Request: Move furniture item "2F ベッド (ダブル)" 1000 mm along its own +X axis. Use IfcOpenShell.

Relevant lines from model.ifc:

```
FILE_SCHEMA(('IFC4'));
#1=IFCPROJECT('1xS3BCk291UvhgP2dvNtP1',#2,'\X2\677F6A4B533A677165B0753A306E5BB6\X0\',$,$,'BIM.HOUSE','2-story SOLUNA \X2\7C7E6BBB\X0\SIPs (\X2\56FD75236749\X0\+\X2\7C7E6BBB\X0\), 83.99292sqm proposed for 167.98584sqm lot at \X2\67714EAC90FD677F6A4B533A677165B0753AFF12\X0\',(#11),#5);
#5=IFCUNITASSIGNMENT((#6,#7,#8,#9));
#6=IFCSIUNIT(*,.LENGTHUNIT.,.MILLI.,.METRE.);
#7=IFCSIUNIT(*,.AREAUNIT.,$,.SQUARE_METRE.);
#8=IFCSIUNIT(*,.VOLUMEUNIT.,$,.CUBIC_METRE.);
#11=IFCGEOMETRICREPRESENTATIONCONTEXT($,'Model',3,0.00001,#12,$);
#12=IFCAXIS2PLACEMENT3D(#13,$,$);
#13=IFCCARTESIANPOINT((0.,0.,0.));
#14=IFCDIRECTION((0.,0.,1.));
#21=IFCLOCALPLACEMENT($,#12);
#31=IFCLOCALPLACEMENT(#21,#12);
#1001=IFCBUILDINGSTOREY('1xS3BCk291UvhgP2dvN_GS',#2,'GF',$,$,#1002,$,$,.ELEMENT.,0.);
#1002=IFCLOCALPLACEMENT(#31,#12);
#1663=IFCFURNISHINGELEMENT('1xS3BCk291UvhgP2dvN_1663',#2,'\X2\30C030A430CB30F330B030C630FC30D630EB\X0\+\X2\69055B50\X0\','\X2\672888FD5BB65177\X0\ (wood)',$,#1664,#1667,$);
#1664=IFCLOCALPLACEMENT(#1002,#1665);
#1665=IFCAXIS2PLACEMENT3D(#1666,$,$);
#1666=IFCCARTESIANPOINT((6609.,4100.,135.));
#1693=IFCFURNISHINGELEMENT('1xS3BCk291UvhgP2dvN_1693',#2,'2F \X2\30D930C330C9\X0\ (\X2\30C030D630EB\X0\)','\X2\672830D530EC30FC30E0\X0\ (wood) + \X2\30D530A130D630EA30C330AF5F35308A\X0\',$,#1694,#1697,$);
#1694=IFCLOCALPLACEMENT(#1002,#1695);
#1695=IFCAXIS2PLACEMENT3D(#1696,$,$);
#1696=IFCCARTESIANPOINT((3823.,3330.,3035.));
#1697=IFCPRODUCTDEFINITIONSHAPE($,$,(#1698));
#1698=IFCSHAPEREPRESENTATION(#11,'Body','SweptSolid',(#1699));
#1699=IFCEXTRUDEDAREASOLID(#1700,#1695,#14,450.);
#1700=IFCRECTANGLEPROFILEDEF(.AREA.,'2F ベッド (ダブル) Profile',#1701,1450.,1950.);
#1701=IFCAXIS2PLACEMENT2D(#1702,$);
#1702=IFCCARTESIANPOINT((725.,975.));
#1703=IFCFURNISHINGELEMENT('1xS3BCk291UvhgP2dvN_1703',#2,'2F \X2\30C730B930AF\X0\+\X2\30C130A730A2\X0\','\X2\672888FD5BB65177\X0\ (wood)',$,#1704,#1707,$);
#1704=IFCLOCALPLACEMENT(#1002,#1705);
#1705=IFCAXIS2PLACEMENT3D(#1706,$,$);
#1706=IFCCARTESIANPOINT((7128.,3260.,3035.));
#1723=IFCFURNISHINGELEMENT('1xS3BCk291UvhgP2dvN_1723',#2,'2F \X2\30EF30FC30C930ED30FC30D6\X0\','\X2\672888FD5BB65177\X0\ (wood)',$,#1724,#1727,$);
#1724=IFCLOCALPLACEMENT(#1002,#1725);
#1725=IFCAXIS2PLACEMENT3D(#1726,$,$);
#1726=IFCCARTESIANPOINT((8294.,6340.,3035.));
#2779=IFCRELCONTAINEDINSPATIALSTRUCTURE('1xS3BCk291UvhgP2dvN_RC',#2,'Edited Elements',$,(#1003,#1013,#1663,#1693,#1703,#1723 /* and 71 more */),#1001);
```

```python
import ifcopenshell
import ifcopenshell.api.geometry
import ifcopenshell.util.placement
import ifcopenshell.util.unit

model = ifcopenshell.open("model.ifc")
unit_scale = ifcopenshell.util.unit.calculate_unit_scale(model)

item = model.by_guid("1xS3BCk291UvhgP2dvN_1693")
matrix = ifcopenshell.util.placement.get_local_placement(item.ObjectPlacement)
matrix[:3, 3] += matrix[:3, 0] * 1 / unit_scale
ifcopenshell.api.geometry.edit_object_placement(model, product=item, matrix=matrix, is_si=False)

print(ifcopenshell.util.placement.get_local_placement(item.ObjectPlacement).round(3) + 0.0)

model.write("model_edited.ifc")
```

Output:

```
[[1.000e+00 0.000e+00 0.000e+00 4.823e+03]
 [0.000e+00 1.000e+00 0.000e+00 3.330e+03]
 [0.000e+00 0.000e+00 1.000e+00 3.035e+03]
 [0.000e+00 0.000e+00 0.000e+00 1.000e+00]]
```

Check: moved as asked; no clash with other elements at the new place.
